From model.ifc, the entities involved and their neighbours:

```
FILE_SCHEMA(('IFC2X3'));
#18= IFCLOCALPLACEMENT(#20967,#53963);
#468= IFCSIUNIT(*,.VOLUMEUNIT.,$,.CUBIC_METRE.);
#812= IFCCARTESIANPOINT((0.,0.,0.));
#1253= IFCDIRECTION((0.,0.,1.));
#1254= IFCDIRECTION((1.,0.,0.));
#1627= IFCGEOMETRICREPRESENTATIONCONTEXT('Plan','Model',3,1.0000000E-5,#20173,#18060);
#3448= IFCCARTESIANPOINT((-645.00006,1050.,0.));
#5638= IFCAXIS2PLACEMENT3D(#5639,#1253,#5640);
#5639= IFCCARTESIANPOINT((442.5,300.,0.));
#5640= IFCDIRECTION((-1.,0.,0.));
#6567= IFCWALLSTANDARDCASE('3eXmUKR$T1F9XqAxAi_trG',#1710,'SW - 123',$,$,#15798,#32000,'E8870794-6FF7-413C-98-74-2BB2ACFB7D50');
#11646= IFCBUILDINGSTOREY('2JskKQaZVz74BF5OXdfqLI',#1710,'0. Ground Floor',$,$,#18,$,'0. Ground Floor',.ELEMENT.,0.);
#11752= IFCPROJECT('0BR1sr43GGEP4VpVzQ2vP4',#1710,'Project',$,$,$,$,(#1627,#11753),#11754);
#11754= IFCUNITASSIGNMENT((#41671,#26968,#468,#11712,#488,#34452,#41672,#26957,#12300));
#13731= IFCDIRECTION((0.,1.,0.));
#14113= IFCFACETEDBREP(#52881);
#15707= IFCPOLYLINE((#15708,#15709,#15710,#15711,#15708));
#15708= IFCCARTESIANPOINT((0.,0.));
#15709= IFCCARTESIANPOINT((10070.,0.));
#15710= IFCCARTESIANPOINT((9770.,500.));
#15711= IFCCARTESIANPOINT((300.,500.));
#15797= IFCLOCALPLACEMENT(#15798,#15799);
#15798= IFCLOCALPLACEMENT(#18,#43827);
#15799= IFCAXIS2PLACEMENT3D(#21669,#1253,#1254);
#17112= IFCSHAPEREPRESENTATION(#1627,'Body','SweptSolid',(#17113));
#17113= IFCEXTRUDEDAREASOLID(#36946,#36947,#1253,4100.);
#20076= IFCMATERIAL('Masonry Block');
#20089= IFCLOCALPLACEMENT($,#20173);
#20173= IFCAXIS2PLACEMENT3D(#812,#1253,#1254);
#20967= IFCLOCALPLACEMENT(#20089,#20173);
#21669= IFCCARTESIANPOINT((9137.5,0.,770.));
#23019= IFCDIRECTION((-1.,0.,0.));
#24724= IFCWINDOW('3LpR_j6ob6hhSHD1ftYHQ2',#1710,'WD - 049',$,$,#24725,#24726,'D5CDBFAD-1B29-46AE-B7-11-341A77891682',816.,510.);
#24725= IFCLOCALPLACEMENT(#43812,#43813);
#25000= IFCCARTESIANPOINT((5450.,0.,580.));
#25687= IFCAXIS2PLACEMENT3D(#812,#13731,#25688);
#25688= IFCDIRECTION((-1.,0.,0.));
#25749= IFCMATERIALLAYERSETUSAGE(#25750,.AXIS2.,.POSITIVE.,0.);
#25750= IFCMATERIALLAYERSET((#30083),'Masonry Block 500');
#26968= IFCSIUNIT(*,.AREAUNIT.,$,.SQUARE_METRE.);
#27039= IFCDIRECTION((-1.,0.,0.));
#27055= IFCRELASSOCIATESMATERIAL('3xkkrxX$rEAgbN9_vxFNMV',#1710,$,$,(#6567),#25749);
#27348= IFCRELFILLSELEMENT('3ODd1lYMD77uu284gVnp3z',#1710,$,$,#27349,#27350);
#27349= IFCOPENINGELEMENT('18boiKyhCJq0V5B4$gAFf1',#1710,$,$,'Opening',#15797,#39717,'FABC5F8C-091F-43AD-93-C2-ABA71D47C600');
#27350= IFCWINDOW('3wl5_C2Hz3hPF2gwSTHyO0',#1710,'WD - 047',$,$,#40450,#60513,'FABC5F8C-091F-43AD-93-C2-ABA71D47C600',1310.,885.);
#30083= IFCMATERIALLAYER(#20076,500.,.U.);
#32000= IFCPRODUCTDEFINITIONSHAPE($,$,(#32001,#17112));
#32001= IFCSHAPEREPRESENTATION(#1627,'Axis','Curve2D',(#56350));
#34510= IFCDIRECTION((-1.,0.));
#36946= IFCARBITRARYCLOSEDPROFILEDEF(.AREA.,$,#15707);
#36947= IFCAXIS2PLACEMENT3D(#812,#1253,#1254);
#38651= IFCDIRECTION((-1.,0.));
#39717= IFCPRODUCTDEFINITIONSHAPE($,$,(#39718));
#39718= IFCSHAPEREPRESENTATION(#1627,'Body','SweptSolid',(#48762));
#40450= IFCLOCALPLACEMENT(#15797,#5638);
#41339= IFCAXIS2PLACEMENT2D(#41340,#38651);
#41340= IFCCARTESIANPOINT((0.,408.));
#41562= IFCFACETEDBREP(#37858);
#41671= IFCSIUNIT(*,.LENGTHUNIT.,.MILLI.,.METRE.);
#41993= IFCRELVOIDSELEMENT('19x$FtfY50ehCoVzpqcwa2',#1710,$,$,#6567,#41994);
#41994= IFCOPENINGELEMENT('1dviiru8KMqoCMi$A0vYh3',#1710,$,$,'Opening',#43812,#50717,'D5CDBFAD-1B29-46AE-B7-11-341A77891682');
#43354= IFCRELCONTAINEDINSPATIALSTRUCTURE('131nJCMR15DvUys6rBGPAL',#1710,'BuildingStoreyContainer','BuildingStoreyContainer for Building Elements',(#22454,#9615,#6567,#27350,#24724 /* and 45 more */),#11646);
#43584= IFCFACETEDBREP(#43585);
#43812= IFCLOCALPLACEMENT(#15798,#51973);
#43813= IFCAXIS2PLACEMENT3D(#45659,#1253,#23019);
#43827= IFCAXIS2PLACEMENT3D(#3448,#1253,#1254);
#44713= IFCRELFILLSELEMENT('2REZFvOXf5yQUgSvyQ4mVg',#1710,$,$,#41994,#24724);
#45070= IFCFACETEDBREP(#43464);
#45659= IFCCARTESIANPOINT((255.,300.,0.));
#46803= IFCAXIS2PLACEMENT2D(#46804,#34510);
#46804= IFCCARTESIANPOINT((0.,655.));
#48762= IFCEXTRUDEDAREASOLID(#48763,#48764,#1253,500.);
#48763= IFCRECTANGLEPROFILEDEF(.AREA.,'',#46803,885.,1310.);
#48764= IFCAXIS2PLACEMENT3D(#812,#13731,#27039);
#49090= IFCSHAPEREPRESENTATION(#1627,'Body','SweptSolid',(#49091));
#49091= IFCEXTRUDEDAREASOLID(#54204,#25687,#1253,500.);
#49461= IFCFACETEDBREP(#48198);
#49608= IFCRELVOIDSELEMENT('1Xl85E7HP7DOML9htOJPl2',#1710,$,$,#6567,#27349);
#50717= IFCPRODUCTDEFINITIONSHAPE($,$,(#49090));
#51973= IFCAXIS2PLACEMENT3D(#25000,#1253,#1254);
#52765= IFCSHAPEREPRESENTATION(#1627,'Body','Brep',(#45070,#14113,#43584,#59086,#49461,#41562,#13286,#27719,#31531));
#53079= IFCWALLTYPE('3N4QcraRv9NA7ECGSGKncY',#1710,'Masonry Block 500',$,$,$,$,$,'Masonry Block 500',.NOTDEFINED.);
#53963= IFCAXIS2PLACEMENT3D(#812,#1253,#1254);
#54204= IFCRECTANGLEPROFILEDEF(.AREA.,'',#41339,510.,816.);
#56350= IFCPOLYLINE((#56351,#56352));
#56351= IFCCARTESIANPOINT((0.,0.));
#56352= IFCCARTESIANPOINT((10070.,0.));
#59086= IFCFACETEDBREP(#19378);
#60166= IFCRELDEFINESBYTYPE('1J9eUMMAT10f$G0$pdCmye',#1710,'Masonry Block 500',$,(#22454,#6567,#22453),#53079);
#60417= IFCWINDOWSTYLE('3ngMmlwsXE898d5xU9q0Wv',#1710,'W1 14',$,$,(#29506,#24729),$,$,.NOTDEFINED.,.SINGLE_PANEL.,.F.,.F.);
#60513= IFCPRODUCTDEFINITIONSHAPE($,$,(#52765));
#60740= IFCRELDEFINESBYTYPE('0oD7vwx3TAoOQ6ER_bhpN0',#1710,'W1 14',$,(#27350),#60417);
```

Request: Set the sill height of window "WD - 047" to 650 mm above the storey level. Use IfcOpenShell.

```python
import numpy as np
import ifcopenshell
import ifcopenshell.api.geometry
import ifcopenshell.geom
import ifcopenshell.util.element
import ifcopenshell.util.placement
import ifcopenshell.util.shape
import ifcopenshell.util.unit

model = ifcopenshell.open("model.ifc")
unit_scale = ifcopenshell.util.unit.calculate_unit_scale(model)

window = model.by_guid("3wl5_C2Hz3hPF2gwSTHyO0")
opening = window.FillsVoids[0].RelatingOpeningElement
storey = ifcopenshell.util.element.get_container(window, ifc_class="IfcBuildingStorey")
level = ifcopenshell.util.placement.get_local_placement(storey.ObjectPlacement)[2, 3]

# The opening's origin need not be at the sill, so measure its lowest point.
shape = ifcopenshell.geom.create_shape(ifcopenshell.geom.settings(), opening)
bottom = ifcopenshell.util.shape.get_shape_bottom_elevation(shape, shape.geometry) / unit_scale
dz = level + 650.0 - bottom

shift = np.array([0.0, 0.0, dz])
# The window is placed relative to its opening, so it follows when the opening moves.
matrix = ifcopenshell.util.placement.get_local_placement(opening.ObjectPlacement)
matrix[:3, 3] += shift
ifcopenshell.api.geometry.edit_object_placement(
    model, product=opening, matrix=matrix, is_si=False, should_transform_children=True
)

print(f"moved by {dz * unit_scale:+.3f} m")

model.write("model-out.ifc")
```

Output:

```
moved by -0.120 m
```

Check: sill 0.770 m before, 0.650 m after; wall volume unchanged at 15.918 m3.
